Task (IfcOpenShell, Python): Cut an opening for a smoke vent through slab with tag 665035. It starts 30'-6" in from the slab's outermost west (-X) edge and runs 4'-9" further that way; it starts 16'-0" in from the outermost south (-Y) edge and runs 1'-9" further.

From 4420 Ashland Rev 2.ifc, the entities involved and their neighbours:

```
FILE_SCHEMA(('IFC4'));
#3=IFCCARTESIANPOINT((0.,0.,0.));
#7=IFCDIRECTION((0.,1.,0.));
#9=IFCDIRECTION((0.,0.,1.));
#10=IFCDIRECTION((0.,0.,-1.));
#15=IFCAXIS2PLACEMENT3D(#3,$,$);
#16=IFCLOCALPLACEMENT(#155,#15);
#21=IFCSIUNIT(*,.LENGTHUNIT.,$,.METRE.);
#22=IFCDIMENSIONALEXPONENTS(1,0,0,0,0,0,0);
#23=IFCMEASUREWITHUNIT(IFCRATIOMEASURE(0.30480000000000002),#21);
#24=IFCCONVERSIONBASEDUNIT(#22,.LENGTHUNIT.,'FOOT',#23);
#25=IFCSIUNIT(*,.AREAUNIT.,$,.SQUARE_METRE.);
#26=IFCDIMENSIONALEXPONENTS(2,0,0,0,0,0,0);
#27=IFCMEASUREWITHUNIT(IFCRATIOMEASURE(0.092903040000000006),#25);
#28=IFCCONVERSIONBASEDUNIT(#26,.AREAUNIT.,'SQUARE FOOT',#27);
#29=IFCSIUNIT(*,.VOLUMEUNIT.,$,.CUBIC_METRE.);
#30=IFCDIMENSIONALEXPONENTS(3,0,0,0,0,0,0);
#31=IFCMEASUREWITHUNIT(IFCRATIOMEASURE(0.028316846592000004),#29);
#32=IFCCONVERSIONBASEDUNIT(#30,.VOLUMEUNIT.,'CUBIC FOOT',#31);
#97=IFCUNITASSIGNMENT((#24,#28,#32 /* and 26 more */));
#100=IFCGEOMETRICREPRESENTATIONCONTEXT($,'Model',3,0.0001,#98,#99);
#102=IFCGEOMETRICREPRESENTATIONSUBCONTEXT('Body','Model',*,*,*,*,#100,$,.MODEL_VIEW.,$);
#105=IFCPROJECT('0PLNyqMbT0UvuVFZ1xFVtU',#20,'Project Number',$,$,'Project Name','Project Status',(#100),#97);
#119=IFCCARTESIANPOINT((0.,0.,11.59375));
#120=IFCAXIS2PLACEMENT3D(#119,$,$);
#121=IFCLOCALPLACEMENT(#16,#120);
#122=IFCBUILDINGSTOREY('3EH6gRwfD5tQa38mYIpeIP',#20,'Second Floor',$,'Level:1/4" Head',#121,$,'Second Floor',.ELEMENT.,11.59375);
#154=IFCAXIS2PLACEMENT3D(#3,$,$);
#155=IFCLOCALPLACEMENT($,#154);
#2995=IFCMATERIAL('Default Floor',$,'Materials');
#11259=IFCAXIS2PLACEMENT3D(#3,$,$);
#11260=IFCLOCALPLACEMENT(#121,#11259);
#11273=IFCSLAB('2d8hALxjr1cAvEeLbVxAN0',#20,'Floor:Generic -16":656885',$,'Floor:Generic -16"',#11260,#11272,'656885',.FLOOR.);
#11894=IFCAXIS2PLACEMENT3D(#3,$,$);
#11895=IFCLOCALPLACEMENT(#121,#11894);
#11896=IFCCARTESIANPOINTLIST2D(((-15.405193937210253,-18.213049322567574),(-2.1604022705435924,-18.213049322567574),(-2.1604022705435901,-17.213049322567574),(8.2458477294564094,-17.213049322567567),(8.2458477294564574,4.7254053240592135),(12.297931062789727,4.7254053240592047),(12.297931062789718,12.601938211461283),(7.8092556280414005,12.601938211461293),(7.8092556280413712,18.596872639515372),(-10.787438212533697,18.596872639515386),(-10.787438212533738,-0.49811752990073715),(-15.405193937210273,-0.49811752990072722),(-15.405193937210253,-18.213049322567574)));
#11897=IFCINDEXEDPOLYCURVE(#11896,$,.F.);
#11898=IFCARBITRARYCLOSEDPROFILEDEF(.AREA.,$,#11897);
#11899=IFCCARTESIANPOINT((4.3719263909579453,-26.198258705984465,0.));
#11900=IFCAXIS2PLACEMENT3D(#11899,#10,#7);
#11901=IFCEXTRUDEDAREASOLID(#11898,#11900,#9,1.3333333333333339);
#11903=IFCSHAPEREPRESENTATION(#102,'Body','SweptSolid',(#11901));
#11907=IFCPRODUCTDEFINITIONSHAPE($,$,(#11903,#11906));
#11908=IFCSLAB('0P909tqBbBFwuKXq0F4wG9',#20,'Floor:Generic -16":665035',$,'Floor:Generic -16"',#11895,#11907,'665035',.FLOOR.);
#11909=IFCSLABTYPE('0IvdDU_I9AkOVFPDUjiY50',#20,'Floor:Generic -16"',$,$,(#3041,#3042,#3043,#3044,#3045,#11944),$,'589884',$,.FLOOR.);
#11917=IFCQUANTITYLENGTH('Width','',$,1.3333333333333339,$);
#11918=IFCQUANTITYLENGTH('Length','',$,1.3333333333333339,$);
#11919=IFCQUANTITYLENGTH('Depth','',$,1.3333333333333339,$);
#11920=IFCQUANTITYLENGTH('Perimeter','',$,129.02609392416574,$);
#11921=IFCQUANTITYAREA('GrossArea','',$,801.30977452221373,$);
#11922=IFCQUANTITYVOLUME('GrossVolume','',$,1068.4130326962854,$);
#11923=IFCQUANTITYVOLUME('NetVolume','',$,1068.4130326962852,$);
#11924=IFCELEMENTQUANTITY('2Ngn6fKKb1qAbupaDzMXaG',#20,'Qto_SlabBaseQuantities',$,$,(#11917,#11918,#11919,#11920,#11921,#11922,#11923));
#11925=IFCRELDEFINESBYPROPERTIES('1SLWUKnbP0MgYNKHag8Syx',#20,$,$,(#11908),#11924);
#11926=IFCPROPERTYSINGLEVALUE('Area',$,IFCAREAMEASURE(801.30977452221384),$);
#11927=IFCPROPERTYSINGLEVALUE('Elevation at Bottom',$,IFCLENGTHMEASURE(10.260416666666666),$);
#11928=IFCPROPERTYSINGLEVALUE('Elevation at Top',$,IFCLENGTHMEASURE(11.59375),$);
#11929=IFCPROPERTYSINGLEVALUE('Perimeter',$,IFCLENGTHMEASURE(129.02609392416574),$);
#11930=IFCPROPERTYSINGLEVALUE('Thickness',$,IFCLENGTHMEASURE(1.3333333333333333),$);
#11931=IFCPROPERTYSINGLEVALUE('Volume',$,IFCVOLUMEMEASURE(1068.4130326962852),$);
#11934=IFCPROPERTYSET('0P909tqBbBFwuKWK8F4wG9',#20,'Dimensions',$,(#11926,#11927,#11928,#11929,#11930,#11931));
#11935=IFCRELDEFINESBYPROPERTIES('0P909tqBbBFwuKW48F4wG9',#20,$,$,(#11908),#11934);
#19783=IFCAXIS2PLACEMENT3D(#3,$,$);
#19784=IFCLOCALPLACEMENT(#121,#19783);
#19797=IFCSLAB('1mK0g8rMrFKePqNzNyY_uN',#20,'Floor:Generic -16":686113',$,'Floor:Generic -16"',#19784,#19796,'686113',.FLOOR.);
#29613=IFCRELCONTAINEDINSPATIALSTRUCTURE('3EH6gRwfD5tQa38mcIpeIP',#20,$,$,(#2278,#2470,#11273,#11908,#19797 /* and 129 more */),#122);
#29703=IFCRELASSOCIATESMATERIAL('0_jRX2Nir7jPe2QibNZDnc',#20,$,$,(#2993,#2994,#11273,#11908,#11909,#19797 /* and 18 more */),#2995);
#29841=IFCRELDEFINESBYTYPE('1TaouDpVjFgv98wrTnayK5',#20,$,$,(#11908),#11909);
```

```python
import numpy as np
import ifcopenshell
import ifcopenshell.api.feature
import ifcopenshell.api.geometry
import ifcopenshell.api.pset
import ifcopenshell.api.root
import ifcopenshell.geom
import ifcopenshell.util.element
import ifcopenshell.util.placement
import ifcopenshell.util.representation
import ifcopenshell.util.shape
import ifcopenshell.util.unit

model = ifcopenshell.open("4420 Ashland Rev 2.ifc")
unit_scale = ifcopenshell.util.unit.calculate_unit_scale(model)
area_scale = ifcopenshell.util.unit.calculate_unit_scale(model, "AREAUNIT")
volume_scale = ifcopenshell.util.unit.calculate_unit_scale(model, "VOLUMEUNIT")
settings = ifcopenshell.geom.settings()


def volume(element):
    """Net volume in cubic metres, openings subtracted."""
    shape = ifcopenshell.geom.create_shape(settings, element)
    return ifcopenshell.util.shape.get_volume(shape.geometry)


slab = model.by_id(11908)
before = volume(slab)

# Extent in the slab's own axes, in metres. The edges named are its -X and -Y sides.
slab_shape = ifcopenshell.geom.create_shape(settings, slab)
vertices = ifcopenshell.util.shape.get_vertices(slab_shape.geometry)
x_min, y_min, bottom = vertices.min(axis=0)
top = vertices[:, 2].max()

opening = ifcopenshell.api.root.create_entity(model, ifc_class="IfcOpeningElement", name="Smoke vent opening", predefined_type="OPENING")
context = ifcopenshell.util.representation.get_context(model, "Model", "Body", "MODEL_VIEW")
width, depth = 1.4478, 0.5334
outline = [(0.0, 0.0), (width, 0.0), (width, depth), (0.0, depth), (0.0, 0.0)]
# Overshoot both faces by 50 mm so the cut is clean.
shape = ifcopenshell.api.geometry.add_slab_representation(
    model, context=context, depth=top - bottom + 0.1, polyline=outline
)
ifcopenshell.api.geometry.assign_representation(model, product=opening, representation=shape)

matrix = ifcopenshell.util.placement.get_local_placement(slab.ObjectPlacement)
matrix[:, 3] = matrix @ np.append(np.array([x_min + 9.2964, y_min + 4.8768, bottom - 0.05]) / unit_scale, 1.0)
ifcopenshell.api.geometry.edit_object_placement(model, product=opening, matrix=matrix, is_si=False)
ifcopenshell.api.feature.add_feature(model, feature=opening, element=slab)

after = volume(slab)

# Update the slab's stored quantities.
qto = model.by_id(ifcopenshell.util.element.get_pset(slab, "Qto_SlabBaseQuantities", should_inherit=False)["id"])
ifcopenshell.api.pset.edit_qto(model, qto=qto, properties={"NetVolume": after / volume_scale})
pset = model.by_id(ifcopenshell.util.element.get_pset(slab, "Dimensions", should_inherit=False)["id"])
ifcopenshell.api.pset.edit_pset(model, pset=pset, properties={
    "Area": model.create_entity("IfcAreaMeasure", after / (top - bottom) / area_scale),
    "Volume": model.create_entity("IfcVolumeMeasure", after / volume_scale),
})

print(f"slab volume {before:.3f} -> {after:.3f} m3")

model.write("4420 Ashland Rev 2_edited.ifc")
```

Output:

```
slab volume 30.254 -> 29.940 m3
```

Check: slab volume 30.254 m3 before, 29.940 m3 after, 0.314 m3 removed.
